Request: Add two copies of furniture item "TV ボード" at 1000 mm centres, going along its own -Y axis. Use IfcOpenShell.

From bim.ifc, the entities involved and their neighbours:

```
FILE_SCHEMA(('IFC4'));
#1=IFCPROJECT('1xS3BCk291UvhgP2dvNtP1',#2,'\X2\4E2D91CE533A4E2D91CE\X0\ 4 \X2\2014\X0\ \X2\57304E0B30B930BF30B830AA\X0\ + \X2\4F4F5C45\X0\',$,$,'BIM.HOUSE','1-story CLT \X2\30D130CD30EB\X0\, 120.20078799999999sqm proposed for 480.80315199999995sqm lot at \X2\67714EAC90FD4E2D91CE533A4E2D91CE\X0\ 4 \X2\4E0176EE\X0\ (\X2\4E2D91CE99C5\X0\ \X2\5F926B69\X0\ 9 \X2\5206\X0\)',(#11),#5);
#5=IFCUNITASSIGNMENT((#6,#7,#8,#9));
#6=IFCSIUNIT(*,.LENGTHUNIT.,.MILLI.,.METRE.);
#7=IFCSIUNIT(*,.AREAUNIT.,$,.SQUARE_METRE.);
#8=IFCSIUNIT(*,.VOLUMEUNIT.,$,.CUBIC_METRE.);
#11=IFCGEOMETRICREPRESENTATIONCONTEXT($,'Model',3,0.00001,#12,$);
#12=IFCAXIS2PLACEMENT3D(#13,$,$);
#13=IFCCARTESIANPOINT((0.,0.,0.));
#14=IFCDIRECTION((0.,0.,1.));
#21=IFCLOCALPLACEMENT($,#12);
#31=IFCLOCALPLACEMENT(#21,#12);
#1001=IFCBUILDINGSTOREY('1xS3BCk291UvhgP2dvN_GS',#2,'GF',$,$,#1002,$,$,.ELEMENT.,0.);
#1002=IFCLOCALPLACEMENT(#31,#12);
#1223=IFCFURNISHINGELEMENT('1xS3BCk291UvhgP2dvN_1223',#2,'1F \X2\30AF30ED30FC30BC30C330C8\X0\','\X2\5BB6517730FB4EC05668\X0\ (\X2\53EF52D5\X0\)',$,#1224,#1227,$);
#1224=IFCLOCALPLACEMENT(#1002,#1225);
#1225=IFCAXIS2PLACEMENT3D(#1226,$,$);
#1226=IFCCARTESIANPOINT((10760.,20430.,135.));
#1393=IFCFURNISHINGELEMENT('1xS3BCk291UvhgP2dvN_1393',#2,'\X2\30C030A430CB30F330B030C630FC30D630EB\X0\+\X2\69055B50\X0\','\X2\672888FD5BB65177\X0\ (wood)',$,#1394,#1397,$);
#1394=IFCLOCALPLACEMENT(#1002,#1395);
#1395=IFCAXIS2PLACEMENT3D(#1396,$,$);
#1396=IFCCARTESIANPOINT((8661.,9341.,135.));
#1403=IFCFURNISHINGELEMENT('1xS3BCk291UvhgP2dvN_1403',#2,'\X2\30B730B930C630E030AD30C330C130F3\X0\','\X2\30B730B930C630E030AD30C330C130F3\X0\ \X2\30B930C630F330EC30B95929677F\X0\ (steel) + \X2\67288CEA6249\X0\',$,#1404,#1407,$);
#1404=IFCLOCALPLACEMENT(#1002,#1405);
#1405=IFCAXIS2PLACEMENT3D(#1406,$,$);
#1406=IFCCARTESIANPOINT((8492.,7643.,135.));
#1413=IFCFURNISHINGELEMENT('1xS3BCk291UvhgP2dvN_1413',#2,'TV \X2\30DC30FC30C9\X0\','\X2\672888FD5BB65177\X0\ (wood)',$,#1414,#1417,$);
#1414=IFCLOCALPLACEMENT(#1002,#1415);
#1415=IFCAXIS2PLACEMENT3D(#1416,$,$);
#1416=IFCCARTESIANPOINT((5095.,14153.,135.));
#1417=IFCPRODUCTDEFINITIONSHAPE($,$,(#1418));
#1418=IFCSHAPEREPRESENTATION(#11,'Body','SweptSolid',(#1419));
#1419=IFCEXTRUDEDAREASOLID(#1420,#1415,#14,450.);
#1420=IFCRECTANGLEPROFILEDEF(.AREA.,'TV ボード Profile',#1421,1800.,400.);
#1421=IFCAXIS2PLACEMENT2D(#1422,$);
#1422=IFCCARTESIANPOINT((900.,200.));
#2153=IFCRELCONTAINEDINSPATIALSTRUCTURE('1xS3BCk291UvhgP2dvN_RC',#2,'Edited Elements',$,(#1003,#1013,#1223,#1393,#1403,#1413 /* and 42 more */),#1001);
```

```python
import ifcopenshell
import ifcopenshell.api.geometry
import ifcopenshell.api.root
import ifcopenshell.util.element
import ifcopenshell.util.placement

model = ifcopenshell.open("bim.ifc")


def reuse_history(source, copy):
    """copy_class also copies each property set's owner history, people and application; keep the originals."""
    for rel in copy.IsDefinedBy:
        if rel.is_a("IfcRelDefinesByProperties") and (history := rel.RelatingPropertyDefinition.OwnerHistory):
            rel.RelatingPropertyDefinition.OwnerHistory = source.OwnerHistory
            ifcopenshell.util.element.remove_deep2(model, history)


source = model.by_id(1413)
base = ifcopenshell.util.placement.get_local_placement(source.ObjectPlacement)
step = -base[:3, 1] * 1000.0

for i in range(1, 3):
    copy = ifcopenshell.api.root.copy_class(model, product=source)
    copy.Representation = ifcopenshell.util.element.copy_deep(
        model, source.Representation, exclude=["IfcGeometricRepresentationContext", "IfcRepresentationMap"]
    )
    reuse_history(source, copy)
    matrix = base.copy()
    matrix[:3, 3] += i * step
    print("added at", matrix[:3, 3].round(3) + 0.0)
    ifcopenshell.api.geometry.edit_object_placement(model, product=copy, matrix=matrix, is_si=False)

model.write("bim_v2.ifc")
```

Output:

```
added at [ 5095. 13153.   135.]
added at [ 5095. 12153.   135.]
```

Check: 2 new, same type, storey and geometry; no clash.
